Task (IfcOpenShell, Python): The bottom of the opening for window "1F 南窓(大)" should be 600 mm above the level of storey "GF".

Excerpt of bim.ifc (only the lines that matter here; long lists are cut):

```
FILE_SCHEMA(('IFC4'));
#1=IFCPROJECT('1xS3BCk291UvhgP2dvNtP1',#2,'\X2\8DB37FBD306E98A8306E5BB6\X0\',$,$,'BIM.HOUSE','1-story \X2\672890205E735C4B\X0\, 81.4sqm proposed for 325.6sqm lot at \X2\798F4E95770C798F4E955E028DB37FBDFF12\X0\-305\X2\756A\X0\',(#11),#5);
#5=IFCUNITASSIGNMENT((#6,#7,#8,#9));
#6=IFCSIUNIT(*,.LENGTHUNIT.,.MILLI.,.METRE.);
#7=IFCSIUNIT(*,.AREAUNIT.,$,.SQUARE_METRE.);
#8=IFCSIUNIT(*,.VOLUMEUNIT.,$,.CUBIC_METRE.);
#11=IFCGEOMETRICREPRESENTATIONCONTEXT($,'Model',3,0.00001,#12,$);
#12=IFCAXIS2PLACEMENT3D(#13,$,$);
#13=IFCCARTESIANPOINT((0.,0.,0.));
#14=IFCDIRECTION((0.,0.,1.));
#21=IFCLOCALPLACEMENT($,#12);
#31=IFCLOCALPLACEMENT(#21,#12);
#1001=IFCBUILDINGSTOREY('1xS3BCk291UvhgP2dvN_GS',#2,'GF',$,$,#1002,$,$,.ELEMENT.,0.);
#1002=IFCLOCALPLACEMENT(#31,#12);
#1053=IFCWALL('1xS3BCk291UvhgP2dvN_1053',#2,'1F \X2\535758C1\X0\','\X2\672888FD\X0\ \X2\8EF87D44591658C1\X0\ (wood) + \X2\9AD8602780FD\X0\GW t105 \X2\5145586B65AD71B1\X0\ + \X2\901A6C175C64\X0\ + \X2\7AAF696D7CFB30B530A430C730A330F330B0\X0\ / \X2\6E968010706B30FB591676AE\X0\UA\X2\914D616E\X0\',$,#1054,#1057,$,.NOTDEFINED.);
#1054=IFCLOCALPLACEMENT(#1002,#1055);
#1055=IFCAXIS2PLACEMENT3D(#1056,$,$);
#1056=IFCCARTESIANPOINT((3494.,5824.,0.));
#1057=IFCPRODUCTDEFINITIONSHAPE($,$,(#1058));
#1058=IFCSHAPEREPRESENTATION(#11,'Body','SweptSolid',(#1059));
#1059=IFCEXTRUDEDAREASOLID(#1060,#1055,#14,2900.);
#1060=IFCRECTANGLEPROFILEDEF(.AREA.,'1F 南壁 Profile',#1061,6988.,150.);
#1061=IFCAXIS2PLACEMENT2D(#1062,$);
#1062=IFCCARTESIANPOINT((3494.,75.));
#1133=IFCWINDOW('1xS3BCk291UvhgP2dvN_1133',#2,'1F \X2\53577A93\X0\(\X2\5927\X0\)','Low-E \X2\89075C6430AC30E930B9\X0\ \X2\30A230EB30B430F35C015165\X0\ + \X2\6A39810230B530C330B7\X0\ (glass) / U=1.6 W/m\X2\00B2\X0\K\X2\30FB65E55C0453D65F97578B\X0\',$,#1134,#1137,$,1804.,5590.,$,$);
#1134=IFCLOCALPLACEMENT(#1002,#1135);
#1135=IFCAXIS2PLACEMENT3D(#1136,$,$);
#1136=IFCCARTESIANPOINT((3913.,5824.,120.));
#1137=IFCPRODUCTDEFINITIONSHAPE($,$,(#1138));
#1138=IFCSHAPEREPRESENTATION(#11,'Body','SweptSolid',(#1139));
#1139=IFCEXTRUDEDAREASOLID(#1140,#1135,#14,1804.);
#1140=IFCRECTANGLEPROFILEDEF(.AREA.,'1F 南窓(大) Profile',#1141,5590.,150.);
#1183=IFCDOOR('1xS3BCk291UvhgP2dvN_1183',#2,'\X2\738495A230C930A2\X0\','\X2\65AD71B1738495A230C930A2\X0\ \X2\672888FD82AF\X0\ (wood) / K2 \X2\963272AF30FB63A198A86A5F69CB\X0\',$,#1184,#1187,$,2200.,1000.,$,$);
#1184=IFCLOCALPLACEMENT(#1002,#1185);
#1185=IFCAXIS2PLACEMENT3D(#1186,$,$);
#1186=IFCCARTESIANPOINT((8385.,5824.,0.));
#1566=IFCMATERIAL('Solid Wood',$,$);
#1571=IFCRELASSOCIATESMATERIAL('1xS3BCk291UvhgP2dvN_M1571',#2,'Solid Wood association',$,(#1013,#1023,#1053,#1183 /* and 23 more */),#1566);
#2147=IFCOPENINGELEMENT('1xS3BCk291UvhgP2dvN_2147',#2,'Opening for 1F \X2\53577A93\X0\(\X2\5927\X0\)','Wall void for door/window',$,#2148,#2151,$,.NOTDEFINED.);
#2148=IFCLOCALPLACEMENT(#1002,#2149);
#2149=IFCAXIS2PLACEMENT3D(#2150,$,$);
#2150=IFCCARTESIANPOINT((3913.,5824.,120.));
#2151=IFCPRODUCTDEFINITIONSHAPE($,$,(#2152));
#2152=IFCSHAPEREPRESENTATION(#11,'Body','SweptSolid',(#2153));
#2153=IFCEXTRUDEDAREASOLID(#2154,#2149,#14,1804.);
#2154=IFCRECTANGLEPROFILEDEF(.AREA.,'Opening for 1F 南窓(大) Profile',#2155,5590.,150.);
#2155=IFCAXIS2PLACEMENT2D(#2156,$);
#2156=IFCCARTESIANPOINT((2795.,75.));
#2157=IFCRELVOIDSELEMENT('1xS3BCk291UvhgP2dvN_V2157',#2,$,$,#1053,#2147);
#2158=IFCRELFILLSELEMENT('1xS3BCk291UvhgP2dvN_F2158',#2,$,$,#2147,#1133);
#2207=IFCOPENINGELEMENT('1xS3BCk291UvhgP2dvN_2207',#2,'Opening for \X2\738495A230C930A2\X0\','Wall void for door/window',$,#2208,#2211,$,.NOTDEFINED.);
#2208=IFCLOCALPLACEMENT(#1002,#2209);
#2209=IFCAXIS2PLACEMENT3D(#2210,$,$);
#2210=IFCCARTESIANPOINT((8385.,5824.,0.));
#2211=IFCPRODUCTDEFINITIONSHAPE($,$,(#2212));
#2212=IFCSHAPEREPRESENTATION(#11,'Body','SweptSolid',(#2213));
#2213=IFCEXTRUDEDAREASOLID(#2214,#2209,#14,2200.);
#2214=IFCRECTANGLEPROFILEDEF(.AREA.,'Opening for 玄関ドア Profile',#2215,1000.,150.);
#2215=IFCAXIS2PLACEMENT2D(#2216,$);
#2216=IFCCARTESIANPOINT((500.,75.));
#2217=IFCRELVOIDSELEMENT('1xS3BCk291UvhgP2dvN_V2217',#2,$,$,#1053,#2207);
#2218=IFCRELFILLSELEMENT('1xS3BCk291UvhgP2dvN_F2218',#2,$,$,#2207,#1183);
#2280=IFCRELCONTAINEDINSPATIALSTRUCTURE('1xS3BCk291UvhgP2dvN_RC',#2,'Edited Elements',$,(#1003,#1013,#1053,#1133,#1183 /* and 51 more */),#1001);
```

```python
import numpy as np
import ifcopenshell
import ifcopenshell.api.geometry
import ifcopenshell.geom
import ifcopenshell.util.element
import ifcopenshell.util.placement
import ifcopenshell.util.shape
import ifcopenshell.util.unit

model = ifcopenshell.open("bim.ifc")
unit_scale = ifcopenshell.util.unit.calculate_unit_scale(model)

window = model.by_guid("1xS3BCk291UvhgP2dvN_1133")
opening = window.FillsVoids[0].RelatingOpeningElement
storey = ifcopenshell.util.element.get_container(window, ifc_class="IfcBuildingStorey")
level = ifcopenshell.util.placement.get_local_placement(storey.ObjectPlacement)[2, 3]

# The opening's origin need not be at the sill, so measure its lowest point.
shape = ifcopenshell.geom.create_shape(ifcopenshell.geom.settings(), opening)
bottom = ifcopenshell.util.shape.get_shape_bottom_elevation(shape, shape.geometry) / unit_scale
dz = level + 0.6 / unit_scale - bottom

shift = np.array([0.0, 0.0, dz])
# The window is not placed relative to its opening, so move both.
for product in (opening, window):
    matrix = ifcopenshell.util.placement.get_local_placement(product.ObjectPlacement)
    matrix[:3, 3] += shift
    ifcopenshell.api.geometry.edit_object_placement(model, product=product, matrix=matrix, is_si=False)

print(f"moved by {dz * unit_scale:+.3f} m")

model.write("bim_updated.ifc")
```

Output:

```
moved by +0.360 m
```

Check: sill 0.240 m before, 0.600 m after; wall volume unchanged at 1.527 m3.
